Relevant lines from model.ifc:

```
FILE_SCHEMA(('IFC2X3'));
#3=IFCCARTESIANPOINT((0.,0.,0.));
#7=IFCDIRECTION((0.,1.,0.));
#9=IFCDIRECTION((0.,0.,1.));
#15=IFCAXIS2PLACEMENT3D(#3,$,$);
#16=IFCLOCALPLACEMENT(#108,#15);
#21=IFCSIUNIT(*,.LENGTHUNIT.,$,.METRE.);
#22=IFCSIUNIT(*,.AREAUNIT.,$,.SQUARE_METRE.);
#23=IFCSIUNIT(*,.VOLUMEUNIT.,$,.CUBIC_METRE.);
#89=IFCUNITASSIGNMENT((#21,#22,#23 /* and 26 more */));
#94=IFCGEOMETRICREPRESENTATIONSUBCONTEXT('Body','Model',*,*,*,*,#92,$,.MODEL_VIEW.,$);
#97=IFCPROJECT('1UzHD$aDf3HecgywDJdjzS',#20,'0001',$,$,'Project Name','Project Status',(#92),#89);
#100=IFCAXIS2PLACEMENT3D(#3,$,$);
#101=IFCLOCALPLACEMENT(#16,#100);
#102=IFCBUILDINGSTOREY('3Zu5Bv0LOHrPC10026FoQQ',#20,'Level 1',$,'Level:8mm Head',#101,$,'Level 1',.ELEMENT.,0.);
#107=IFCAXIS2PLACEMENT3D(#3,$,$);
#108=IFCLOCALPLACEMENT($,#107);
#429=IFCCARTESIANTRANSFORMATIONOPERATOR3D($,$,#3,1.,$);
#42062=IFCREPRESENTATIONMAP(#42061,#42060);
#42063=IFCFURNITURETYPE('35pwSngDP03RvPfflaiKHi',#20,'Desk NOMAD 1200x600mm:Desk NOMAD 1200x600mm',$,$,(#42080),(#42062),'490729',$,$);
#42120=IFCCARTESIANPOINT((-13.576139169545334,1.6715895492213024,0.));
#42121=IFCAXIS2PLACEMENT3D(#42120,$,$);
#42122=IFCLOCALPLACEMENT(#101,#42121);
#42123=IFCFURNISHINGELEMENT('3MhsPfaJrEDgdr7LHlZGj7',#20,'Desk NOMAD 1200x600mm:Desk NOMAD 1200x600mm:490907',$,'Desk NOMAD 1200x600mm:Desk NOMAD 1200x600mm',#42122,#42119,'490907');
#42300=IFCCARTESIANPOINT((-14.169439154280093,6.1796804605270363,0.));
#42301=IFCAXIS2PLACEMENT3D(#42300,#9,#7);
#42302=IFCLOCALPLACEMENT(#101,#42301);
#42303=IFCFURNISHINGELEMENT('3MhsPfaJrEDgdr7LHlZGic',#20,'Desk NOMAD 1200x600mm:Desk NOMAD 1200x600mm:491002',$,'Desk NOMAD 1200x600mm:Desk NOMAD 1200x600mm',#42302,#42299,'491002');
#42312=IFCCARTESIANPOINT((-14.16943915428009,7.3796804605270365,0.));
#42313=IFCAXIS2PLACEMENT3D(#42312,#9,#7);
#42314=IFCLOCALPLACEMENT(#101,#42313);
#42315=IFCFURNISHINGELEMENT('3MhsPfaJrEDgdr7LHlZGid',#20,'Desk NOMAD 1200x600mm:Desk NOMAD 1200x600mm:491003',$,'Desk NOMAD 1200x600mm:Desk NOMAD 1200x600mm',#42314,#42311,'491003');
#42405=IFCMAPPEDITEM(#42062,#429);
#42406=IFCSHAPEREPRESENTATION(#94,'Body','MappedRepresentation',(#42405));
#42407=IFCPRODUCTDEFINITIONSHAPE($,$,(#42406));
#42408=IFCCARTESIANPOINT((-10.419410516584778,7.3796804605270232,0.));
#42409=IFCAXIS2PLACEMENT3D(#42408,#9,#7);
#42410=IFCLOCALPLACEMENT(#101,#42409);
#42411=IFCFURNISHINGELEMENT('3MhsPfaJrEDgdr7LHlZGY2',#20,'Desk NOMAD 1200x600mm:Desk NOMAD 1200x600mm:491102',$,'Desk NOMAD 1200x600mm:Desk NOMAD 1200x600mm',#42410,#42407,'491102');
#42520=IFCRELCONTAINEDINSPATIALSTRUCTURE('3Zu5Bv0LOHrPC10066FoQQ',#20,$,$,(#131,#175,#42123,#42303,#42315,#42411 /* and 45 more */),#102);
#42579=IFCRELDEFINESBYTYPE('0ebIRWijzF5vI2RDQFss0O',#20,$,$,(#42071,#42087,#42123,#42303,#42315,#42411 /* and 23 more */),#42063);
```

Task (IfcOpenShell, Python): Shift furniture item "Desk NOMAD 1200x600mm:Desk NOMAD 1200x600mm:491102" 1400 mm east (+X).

```python
import ifcopenshell
import ifcopenshell.api.geometry
import ifcopenshell.util.placement
import ifcopenshell.util.unit

model = ifcopenshell.open("model.ifc")
unit_scale = ifcopenshell.util.unit.calculate_unit_scale(model)

item = model.by_guid("3MhsPfaJrEDgdr7LHlZGY2")
matrix = ifcopenshell.util.placement.get_local_placement(item.ObjectPlacement)
matrix[0, 3] += 1.4 / unit_scale
ifcopenshell.api.geometry.edit_object_placement(model, product=item, matrix=matrix, is_si=False)

print(ifcopenshell.util.placement.get_local_placement(item.ObjectPlacement).round(3) + 0.0)

model.write("model_rev.ifc")
```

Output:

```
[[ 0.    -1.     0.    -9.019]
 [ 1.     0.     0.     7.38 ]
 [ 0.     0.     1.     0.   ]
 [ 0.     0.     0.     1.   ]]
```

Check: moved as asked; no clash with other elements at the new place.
